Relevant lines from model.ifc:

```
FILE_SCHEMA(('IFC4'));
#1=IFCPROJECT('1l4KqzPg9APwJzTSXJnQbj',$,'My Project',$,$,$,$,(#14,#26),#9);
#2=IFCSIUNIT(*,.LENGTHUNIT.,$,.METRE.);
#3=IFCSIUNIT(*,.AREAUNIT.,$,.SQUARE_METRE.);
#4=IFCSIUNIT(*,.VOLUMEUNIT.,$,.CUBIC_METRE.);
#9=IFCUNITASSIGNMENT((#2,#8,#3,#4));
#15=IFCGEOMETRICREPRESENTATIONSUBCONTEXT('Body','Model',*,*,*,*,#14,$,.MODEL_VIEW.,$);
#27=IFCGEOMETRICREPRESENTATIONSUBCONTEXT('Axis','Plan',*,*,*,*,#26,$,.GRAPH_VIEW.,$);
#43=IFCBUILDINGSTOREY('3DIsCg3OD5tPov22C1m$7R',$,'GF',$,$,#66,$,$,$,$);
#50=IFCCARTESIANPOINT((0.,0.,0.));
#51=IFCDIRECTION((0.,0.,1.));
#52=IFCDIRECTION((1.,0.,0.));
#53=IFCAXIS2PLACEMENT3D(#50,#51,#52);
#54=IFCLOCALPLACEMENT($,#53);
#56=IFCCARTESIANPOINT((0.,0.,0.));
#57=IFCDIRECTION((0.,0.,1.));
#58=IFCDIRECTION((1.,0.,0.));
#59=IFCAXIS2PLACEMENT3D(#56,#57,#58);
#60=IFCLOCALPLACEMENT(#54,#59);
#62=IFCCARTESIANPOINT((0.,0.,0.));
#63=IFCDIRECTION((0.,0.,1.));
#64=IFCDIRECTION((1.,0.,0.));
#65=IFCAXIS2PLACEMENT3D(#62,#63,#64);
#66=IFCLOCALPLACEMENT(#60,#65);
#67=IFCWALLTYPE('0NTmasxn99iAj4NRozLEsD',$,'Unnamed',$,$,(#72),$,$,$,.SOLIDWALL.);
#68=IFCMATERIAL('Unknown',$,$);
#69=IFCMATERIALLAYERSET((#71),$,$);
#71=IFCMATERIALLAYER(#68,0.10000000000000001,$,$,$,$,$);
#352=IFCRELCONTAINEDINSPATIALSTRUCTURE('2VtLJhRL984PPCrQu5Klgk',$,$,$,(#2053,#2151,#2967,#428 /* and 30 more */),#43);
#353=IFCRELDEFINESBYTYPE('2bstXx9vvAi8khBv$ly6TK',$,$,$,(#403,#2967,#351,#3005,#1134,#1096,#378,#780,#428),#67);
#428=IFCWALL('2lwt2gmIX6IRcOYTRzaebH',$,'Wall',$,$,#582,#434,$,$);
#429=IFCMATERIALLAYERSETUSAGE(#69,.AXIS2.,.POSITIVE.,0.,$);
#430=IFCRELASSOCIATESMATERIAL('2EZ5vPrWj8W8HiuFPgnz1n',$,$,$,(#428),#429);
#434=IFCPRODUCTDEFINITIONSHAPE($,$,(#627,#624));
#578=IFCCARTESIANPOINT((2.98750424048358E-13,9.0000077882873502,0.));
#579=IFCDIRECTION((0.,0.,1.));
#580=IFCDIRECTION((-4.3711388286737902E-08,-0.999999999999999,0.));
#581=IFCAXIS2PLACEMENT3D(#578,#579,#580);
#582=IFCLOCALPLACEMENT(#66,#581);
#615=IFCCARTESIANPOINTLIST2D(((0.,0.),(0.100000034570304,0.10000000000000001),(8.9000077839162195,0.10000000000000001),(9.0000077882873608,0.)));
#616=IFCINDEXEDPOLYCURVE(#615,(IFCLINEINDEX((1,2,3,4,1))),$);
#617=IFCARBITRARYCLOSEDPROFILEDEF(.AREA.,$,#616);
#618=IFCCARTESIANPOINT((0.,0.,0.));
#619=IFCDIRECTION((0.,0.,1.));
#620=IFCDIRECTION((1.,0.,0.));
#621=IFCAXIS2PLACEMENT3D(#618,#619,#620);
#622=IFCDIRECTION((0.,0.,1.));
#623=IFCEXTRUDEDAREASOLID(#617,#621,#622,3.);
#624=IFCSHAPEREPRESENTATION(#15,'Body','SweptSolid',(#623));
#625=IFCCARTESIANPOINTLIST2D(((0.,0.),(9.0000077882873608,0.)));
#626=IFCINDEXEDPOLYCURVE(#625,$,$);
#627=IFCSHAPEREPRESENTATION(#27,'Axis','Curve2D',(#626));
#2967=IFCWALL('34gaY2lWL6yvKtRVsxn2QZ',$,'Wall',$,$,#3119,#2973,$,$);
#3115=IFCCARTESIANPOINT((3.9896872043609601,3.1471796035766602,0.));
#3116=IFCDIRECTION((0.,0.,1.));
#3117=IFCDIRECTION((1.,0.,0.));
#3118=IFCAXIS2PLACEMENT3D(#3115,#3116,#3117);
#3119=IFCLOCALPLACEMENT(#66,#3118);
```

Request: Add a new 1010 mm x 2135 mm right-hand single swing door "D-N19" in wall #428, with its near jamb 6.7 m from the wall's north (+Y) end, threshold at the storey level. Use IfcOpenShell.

```python
import numpy as np
import ifcopenshell
import ifcopenshell.api.feature
import ifcopenshell.api.geometry
import ifcopenshell.api.root
import ifcopenshell.api.spatial
import ifcopenshell.geom
import ifcopenshell.util.element
import ifcopenshell.util.placement
import ifcopenshell.util.representation
import ifcopenshell.util.shape
import ifcopenshell.util.unit

model = ifcopenshell.open("model.ifc")
unit_scale = ifcopenshell.util.unit.calculate_unit_scale(model)
settings = ifcopenshell.geom.settings()


def volume(element):
    """Net volume in cubic metres, openings subtracted."""
    shape = ifcopenshell.geom.create_shape(settings, element)
    return ifcopenshell.util.shape.get_volume(shape.geometry)


wall = model.by_guid("2lwt2gmIX6IRcOYTRzaebH")
storey = ifcopenshell.util.element.get_container(wall, ifc_class="IfcBuildingStorey")
context = ifcopenshell.util.representation.get_context(model, "Model", "Body", "MODEL_VIEW")
before = volume(wall)

width, height, from_end, sill = 1.01, 2.135, 6.7, 0.0  # metres

# The wall runs along its own X axis, and the end named is its -X end.
wall_shape = ifcopenshell.geom.create_shape(settings, wall)
x, y, z = ifcopenshell.util.shape.get_vertices(wall_shape.geometry).T
start = x.min() + from_end
face, thickness = float(y.min()), float(y.max() - y.min())
wall_matrix = ifcopenshell.util.placement.get_local_placement(wall.ObjectPlacement)
level = ifcopenshell.util.placement.get_local_placement(storey.ObjectPlacement)[2, 3]


def in_wall(x, y):
    """Placement at x, y metres in the wall's axes, at sill height."""
    matrix = wall_matrix.copy()
    matrix[:, 3] = wall_matrix @ np.array([x / unit_scale, y / unit_scale, 0.0, 1.0])
    matrix[2, 3] = level + sill / unit_scale
    return matrix


# Opening: a box that overshoots both wall faces by 50 mm.
opening = ifcopenshell.api.root.create_entity(model, ifc_class="IfcOpeningElement", predefined_type="OPENING")
box = ifcopenshell.api.geometry.add_wall_representation(
    model, context=context, length=width, height=height, thickness=thickness + 0.1
)
ifcopenshell.api.geometry.assign_representation(model, product=opening, representation=box)
ifcopenshell.api.geometry.edit_object_placement(model, product=opening, matrix=in_wall(start, face - 0.05), is_si=False)
ifcopenshell.api.feature.add_feature(model, feature=opening, element=wall)

door = ifcopenshell.api.root.create_entity(model, ifc_class="IfcDoor", name="D-N19", predefined_type="DOOR")
door.OverallWidth, door.OverallHeight = width / unit_scale, height / unit_scale
door.OperationType = "SINGLE_SWING_RIGHT"
body = ifcopenshell.api.geometry.add_door_representation(
    model,
    context=context,
    overall_width=door.OverallWidth,
    overall_height=door.OverallHeight,
    operation_type="SINGLE_SWING_RIGHT",
    lining_properties={"LiningDepth": thickness / unit_scale, "ThresholdDepth": thickness / unit_scale},
)
ifcopenshell.api.geometry.assign_representation(model, product=door, representation=body)
ifcopenshell.api.spatial.assign_container(model, products=[door], relating_structure=storey)
ifcopenshell.api.feature.add_filling(model, opening=opening, element=door)

# The lining spans the wall, so the door starts at the wall face.
ifcopenshell.api.geometry.edit_object_placement(model, product=door, matrix=in_wall(start, face), is_si=False)

after = volume(wall)

print(f"wall volume {before:.3f} -> {after:.3f} m3")

model.write("model-out.ifc")
```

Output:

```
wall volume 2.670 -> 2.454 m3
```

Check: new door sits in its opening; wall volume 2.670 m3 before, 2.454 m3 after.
